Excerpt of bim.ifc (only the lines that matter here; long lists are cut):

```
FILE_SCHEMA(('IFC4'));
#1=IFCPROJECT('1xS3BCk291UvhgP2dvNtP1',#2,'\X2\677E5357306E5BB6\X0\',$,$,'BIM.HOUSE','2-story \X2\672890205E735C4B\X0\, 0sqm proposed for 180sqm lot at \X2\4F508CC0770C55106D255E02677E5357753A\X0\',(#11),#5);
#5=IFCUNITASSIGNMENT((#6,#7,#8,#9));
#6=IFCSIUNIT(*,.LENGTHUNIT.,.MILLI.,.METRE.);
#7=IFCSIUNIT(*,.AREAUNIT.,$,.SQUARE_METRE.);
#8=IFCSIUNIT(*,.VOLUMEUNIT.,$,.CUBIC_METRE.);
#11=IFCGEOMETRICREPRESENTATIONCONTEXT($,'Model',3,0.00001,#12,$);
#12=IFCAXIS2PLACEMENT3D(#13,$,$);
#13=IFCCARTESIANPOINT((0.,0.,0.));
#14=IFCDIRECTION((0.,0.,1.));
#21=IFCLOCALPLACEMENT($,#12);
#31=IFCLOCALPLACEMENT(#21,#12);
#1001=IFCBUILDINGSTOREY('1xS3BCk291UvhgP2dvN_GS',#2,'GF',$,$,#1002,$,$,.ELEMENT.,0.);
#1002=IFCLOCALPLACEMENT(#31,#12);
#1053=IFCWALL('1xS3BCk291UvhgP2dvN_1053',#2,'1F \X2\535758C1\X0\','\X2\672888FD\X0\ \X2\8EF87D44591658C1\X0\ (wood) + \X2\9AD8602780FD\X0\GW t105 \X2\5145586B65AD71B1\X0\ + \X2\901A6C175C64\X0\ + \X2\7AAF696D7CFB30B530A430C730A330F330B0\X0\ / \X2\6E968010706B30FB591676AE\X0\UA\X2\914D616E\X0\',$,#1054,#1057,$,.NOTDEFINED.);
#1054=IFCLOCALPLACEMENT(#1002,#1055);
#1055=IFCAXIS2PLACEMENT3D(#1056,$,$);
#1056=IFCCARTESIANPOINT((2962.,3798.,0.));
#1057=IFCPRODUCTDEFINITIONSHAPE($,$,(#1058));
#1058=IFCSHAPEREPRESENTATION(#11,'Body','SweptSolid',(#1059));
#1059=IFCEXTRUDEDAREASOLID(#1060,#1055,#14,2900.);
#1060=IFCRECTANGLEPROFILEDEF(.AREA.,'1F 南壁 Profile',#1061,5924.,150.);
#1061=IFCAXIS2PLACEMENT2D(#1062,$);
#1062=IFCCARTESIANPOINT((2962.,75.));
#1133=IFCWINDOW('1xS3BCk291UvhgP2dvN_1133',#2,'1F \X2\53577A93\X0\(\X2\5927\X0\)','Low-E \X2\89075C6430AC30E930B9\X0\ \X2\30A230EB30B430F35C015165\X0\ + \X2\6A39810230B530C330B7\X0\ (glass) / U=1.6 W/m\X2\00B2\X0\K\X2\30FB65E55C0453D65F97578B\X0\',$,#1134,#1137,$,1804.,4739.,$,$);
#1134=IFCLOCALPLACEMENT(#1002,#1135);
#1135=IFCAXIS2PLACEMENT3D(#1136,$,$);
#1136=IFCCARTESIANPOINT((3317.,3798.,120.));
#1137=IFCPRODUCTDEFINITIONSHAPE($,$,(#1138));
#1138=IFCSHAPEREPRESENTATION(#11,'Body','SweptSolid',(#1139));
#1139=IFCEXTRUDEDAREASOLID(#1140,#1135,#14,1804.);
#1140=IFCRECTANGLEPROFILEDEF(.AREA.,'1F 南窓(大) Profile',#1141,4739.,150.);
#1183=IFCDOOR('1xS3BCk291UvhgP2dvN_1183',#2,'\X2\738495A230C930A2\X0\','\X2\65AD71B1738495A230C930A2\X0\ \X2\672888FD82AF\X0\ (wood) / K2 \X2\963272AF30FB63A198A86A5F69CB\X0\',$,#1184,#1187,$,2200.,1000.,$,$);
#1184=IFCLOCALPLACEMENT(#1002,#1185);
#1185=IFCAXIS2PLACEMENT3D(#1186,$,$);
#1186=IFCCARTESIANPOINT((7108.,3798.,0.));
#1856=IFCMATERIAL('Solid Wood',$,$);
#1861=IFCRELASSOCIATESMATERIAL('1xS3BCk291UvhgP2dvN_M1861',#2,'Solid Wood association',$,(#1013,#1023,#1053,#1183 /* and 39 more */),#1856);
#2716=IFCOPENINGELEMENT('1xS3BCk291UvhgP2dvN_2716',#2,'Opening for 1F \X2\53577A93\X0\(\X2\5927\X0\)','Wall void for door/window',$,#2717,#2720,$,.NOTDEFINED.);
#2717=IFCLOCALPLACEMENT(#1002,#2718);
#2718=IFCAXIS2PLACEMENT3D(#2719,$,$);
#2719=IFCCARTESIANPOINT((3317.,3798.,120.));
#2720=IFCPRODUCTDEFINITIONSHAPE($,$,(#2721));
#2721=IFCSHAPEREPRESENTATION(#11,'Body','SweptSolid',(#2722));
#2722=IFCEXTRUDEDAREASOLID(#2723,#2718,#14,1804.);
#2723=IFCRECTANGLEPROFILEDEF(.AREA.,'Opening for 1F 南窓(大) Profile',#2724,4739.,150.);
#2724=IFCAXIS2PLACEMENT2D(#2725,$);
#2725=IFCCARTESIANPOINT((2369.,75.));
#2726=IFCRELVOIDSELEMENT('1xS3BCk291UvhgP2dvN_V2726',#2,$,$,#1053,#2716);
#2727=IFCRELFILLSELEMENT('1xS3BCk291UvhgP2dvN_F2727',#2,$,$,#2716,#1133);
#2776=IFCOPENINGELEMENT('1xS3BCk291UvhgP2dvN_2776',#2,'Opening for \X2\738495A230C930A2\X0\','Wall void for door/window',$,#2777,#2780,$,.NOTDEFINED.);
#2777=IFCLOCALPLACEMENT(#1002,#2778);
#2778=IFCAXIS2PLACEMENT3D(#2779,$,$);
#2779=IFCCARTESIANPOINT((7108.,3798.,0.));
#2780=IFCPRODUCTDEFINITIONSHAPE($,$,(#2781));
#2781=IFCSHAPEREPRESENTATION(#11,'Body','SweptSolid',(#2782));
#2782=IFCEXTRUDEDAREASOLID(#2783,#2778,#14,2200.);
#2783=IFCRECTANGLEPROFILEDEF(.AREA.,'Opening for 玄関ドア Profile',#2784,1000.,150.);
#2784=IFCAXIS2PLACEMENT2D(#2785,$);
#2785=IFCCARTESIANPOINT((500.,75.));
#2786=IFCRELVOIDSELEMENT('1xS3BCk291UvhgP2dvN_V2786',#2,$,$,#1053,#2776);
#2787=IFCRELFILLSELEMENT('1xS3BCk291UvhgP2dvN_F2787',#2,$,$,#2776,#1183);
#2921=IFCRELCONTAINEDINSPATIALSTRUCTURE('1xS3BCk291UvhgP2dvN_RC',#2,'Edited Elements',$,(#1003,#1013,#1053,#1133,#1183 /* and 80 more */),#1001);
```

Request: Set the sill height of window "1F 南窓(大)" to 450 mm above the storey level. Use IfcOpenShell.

```python
import numpy as np
import ifcopenshell
import ifcopenshell.api.geometry
import ifcopenshell.geom
import ifcopenshell.util.element
import ifcopenshell.util.placement
import ifcopenshell.util.shape
import ifcopenshell.util.unit

model = ifcopenshell.open("bim.ifc")
unit_scale = ifcopenshell.util.unit.calculate_unit_scale(model)

window = model.by_id(1133)
opening = window.FillsVoids[0].RelatingOpeningElement
storey = ifcopenshell.util.element.get_container(window, ifc_class="IfcBuildingStorey")
level = ifcopenshell.util.placement.get_local_placement(storey.ObjectPlacement)[2, 3]

# The opening's origin need not be at the sill, so measure its lowest point.
shape = ifcopenshell.geom.create_shape(ifcopenshell.geom.settings(), opening)
bottom = ifcopenshell.util.shape.get_shape_bottom_elevation(shape, shape.geometry) / unit_scale
dz = level + 0.45 / unit_scale - bottom

shift = np.array([0.0, 0.0, dz])
# The window is not placed relative to its opening, so move both.
for product in (opening, window):
    matrix = ifcopenshell.util.placement.get_local_placement(product.ObjectPlacement)
    matrix[:3, 3] += shift
    ifcopenshell.api.geometry.edit_object_placement(model, product=product, matrix=matrix, is_si=False)

print(f"moved by {dz * unit_scale:+.3f} m")

model.write("bim_rev.ifc")
```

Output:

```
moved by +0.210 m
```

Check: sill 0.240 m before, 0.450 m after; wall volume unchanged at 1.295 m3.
